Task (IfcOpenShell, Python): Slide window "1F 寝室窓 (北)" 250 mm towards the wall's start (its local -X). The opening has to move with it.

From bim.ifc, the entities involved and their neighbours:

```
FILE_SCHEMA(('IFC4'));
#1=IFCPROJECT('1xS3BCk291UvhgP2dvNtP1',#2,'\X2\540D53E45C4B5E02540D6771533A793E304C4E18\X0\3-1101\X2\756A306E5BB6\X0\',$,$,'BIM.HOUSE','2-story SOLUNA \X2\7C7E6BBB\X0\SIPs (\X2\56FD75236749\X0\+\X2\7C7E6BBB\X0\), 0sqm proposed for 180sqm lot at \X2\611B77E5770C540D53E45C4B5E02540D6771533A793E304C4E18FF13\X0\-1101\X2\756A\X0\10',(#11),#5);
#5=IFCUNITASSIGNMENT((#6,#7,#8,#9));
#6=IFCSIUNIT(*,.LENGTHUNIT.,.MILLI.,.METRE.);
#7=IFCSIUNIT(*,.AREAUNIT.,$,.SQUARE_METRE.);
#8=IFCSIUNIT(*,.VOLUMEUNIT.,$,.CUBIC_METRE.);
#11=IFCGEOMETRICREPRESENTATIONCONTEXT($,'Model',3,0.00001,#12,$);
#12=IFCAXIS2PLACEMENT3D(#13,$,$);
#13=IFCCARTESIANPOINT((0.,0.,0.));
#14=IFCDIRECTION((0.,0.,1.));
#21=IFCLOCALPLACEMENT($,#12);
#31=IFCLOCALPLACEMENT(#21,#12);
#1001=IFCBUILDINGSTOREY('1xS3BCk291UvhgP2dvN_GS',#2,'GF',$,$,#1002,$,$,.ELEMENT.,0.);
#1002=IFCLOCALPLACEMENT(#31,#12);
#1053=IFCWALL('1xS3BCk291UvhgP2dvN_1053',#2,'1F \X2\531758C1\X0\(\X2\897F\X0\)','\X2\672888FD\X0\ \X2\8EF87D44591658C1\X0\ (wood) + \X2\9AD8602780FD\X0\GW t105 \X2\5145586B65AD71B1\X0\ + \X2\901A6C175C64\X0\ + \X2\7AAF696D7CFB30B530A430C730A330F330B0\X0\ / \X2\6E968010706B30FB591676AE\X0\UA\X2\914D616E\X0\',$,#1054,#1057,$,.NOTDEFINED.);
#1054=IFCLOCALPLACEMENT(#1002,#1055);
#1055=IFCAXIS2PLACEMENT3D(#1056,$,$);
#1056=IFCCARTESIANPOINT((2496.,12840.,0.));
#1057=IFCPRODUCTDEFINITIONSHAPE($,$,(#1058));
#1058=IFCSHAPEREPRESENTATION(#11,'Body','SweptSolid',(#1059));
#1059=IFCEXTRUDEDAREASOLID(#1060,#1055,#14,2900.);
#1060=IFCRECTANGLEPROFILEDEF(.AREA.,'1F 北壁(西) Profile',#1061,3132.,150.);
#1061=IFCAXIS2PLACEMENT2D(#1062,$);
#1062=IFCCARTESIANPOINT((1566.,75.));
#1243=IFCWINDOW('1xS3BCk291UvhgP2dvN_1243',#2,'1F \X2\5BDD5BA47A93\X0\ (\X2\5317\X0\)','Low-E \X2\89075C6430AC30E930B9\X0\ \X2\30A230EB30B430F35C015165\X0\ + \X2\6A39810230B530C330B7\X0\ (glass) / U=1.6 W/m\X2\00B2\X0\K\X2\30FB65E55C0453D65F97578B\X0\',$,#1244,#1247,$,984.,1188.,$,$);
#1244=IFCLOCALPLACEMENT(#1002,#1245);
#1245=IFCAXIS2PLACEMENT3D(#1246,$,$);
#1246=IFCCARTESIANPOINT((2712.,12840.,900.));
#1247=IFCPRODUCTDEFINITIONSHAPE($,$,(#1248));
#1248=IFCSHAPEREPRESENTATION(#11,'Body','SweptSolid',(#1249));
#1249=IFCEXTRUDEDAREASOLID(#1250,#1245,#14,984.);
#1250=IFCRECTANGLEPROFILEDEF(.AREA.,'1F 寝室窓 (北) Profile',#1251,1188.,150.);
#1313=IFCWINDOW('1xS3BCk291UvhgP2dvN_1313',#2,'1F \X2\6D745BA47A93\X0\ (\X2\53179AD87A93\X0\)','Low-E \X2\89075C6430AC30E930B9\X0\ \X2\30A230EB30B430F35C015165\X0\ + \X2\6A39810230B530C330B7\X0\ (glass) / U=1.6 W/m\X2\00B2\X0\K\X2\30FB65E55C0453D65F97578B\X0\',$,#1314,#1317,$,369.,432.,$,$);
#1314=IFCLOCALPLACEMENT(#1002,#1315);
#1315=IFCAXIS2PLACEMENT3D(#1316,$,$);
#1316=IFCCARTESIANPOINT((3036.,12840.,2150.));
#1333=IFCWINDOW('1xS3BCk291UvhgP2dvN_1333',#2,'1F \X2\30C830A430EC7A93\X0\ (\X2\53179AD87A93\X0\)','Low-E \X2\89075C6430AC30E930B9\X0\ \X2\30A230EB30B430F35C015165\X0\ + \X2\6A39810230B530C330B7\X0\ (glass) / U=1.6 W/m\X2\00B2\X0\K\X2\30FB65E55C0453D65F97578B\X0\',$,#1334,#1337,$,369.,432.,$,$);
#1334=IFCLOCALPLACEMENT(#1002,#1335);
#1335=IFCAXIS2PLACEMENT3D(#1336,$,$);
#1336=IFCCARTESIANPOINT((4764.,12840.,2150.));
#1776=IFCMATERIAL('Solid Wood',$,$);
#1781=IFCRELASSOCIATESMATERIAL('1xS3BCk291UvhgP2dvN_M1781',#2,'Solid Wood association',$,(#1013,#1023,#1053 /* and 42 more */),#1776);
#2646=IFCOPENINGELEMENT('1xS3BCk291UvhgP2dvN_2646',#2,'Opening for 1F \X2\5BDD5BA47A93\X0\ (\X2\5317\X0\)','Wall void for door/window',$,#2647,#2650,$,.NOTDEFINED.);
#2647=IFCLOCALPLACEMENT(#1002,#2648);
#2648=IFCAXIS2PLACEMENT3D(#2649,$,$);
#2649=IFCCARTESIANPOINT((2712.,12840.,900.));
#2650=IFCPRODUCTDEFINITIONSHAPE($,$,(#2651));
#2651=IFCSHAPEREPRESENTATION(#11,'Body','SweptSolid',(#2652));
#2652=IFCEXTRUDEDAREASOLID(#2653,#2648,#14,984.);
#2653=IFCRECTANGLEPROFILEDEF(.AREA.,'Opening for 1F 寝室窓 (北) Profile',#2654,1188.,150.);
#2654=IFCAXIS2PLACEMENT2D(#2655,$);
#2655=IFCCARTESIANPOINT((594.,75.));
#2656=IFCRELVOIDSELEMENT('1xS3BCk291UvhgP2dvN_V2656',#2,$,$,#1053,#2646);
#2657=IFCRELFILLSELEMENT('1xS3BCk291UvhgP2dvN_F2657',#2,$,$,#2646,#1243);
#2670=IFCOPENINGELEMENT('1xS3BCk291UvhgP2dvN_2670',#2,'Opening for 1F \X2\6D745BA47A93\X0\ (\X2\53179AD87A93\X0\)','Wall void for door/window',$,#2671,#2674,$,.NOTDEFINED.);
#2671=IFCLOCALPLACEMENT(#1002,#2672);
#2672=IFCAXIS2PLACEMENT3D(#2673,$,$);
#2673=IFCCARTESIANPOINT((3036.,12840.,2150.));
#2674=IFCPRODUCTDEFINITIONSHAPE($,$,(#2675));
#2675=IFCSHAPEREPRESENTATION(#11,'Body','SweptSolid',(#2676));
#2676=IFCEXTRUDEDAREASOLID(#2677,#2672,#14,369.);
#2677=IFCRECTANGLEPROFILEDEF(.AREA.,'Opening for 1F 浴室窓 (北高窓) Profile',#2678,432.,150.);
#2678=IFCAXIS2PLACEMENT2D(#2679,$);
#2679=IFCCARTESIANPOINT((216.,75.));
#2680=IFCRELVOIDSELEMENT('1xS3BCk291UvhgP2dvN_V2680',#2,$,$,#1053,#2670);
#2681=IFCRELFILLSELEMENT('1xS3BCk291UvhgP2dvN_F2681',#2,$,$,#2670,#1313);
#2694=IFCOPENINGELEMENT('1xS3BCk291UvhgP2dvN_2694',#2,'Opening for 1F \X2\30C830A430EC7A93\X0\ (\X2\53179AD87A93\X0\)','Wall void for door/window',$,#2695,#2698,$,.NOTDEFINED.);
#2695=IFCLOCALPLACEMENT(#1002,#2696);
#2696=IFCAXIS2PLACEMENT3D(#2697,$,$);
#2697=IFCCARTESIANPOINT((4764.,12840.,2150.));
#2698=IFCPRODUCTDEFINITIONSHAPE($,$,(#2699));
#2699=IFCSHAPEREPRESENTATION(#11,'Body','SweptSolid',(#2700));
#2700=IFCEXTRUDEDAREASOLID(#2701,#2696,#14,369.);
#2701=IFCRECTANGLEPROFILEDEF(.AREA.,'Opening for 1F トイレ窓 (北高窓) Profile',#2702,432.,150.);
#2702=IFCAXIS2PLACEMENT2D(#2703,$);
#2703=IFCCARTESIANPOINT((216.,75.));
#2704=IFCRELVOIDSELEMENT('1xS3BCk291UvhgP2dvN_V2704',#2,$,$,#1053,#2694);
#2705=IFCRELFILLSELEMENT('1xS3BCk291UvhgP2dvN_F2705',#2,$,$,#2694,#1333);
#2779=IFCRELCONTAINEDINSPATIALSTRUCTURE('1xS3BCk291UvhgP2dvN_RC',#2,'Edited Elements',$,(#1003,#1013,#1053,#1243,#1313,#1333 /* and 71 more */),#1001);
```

```python
import ifcopenshell
import ifcopenshell.api.geometry
import ifcopenshell.util.placement
import ifcopenshell.util.unit

model = ifcopenshell.open("bim.ifc")
unit_scale = ifcopenshell.util.unit.calculate_unit_scale(model)

window = model.by_id(1243)
opening = window.FillsVoids[0].RelatingOpeningElement
wall = opening.VoidsElements[0].RelatingBuildingElement

wall_matrix = ifcopenshell.util.placement.get_local_placement(wall.ObjectPlacement)
shift = wall_matrix[:3, 0] * -0.25 / unit_scale
before = ifcopenshell.util.placement.get_local_placement(window.ObjectPlacement)[:3, 3].copy()

# The window is not placed relative to its opening, so move both.
for product in (opening, window):
    matrix = ifcopenshell.util.placement.get_local_placement(product.ObjectPlacement)
    matrix[:3, 3] += shift
    ifcopenshell.api.geometry.edit_object_placement(model, product=product, matrix=matrix, is_si=False)

after = ifcopenshell.util.placement.get_local_placement(window.ObjectPlacement)[:3, 3]
print("window moved by", (after - before).round(3) + 0.0)

model.write("bim_edited.ifc")
```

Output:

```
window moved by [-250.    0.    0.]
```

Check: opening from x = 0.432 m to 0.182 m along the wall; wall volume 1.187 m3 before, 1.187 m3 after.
